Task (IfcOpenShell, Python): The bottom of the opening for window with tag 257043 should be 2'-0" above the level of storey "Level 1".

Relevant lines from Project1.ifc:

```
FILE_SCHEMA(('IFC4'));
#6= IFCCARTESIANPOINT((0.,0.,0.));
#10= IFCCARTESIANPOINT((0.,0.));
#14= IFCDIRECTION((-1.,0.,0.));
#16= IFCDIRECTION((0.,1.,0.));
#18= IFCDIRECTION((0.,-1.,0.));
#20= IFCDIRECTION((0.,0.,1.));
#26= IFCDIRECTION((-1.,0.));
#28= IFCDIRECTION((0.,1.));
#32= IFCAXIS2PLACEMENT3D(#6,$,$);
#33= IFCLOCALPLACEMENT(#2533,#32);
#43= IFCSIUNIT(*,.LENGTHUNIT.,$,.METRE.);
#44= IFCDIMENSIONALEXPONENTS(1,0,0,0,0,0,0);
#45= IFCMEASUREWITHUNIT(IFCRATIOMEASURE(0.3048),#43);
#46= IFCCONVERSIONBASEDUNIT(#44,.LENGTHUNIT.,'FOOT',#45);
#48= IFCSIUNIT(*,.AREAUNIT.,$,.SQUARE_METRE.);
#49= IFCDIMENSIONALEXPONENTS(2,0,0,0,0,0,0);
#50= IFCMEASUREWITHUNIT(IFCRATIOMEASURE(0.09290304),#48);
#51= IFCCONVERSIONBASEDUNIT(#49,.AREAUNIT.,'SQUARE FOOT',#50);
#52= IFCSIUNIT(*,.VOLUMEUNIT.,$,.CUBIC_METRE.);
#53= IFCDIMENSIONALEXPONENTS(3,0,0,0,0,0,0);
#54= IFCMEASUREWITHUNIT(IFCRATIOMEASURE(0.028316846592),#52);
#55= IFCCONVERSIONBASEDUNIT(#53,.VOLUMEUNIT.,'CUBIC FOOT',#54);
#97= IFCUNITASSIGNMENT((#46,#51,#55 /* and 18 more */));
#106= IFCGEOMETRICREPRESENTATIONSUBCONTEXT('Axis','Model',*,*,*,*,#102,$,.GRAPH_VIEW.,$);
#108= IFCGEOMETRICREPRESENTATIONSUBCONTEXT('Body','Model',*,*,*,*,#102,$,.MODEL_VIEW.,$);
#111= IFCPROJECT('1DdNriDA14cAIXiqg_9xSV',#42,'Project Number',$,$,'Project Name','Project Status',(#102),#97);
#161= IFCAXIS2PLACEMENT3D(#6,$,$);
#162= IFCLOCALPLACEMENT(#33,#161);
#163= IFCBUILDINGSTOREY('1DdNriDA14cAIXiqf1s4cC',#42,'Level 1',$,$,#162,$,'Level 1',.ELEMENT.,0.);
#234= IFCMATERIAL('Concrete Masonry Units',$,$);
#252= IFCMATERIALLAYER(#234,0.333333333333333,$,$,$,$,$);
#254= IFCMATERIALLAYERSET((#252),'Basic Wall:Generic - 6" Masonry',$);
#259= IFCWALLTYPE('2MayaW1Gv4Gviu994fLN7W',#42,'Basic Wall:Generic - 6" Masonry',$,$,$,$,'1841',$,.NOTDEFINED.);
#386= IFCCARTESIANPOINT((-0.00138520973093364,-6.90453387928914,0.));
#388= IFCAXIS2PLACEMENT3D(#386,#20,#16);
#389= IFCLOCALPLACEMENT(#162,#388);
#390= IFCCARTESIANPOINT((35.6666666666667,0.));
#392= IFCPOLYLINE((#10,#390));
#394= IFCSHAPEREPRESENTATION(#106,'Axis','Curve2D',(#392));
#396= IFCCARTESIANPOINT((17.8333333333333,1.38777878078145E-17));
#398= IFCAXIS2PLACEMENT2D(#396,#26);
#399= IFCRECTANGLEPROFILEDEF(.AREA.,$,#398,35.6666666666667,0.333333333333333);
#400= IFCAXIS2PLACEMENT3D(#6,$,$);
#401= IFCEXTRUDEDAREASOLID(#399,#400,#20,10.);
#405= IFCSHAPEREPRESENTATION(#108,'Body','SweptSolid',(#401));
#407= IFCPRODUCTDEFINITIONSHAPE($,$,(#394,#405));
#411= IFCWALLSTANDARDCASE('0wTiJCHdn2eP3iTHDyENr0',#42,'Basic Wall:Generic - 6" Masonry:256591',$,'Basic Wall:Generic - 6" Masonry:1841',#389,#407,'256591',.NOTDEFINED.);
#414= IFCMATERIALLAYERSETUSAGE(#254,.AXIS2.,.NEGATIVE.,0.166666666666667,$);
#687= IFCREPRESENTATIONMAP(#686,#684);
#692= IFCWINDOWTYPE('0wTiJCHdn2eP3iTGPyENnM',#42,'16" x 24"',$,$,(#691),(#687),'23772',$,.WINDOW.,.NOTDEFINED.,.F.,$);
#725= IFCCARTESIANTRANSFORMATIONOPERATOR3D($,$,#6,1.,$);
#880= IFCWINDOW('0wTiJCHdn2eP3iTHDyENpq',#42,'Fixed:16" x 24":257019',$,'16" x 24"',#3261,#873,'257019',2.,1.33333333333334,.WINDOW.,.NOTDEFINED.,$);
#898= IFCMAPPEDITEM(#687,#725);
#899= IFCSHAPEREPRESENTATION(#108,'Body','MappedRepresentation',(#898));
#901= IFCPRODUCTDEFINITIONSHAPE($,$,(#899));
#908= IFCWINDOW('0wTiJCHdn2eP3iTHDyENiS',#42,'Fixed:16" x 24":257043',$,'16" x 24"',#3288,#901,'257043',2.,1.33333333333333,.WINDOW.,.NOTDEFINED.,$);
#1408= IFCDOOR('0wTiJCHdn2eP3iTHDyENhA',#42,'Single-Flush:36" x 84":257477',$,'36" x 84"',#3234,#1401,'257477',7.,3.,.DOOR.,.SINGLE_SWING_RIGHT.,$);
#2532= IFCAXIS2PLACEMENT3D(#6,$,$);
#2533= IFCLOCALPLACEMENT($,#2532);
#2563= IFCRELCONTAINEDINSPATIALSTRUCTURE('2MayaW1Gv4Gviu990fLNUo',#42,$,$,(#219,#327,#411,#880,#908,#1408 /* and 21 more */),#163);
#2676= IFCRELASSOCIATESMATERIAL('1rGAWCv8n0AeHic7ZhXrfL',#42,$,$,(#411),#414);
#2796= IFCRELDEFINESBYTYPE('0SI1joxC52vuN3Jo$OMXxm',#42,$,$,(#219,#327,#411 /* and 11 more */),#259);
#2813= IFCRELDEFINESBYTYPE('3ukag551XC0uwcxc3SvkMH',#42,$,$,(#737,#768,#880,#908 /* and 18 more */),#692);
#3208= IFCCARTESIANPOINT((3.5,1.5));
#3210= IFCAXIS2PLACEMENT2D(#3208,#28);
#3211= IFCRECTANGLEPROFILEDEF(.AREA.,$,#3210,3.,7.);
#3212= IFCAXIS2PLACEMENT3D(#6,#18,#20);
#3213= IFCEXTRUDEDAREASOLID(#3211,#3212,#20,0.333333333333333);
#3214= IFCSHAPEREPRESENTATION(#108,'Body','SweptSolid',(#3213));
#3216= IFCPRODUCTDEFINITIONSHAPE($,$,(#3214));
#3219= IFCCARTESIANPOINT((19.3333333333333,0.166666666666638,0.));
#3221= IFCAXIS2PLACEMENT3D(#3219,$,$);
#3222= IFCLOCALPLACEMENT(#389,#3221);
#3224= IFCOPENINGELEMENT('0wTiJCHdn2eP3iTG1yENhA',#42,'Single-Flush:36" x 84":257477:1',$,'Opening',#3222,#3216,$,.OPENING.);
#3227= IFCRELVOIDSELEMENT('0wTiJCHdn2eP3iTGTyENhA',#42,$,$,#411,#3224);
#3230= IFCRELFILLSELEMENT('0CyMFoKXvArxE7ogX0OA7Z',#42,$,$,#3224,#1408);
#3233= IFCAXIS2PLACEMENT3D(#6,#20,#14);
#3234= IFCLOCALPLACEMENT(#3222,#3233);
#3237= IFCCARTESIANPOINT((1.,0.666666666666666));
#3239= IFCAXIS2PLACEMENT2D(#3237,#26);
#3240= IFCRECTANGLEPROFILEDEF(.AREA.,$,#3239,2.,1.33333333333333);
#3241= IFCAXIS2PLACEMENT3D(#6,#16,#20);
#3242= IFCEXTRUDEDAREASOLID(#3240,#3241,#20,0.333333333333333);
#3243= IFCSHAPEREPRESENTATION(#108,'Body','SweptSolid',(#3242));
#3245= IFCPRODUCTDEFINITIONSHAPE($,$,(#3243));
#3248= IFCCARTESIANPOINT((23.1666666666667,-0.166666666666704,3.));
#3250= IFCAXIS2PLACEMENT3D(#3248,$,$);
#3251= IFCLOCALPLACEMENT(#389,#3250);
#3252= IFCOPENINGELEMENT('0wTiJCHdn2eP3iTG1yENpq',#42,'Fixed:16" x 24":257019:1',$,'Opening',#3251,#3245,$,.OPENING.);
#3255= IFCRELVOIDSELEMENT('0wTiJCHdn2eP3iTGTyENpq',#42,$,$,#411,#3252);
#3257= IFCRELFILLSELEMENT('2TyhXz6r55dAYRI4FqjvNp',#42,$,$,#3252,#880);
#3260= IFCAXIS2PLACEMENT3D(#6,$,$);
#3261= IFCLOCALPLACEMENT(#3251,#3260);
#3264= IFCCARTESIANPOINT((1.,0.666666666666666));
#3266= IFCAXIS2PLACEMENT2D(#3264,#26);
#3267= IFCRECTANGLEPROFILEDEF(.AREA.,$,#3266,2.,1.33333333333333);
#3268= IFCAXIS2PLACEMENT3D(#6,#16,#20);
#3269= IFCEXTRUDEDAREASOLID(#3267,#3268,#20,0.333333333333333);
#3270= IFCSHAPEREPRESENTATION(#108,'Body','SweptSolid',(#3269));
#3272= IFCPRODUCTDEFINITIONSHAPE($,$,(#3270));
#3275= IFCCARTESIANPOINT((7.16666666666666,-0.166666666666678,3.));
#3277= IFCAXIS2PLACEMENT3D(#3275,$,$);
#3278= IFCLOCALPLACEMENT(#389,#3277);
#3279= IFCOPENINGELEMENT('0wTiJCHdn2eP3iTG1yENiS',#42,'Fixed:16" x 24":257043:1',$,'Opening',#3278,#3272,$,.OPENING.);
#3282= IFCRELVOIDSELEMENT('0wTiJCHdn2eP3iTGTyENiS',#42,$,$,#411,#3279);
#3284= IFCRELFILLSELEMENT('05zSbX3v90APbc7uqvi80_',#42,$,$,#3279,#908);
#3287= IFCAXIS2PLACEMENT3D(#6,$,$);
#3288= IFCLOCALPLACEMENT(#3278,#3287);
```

```python
import numpy as np
import ifcopenshell
import ifcopenshell.api.geometry
import ifcopenshell.geom
import ifcopenshell.util.element
import ifcopenshell.util.placement
import ifcopenshell.util.shape
import ifcopenshell.util.unit

model = ifcopenshell.open("Project1.ifc")
unit_scale = ifcopenshell.util.unit.calculate_unit_scale(model)

window = model.by_id(908)
opening = window.FillsVoids[0].RelatingOpeningElement
storey = ifcopenshell.util.element.get_container(window, ifc_class="IfcBuildingStorey")
level = ifcopenshell.util.placement.get_local_placement(storey.ObjectPlacement)[2, 3]

# The opening's origin need not be at the sill, so measure its lowest point.
shape = ifcopenshell.geom.create_shape(ifcopenshell.geom.settings(), opening)
bottom = ifcopenshell.util.shape.get_shape_bottom_elevation(shape, shape.geometry) / unit_scale
dz = level + 24 * 0.0254 / unit_scale - bottom

shift = np.array([0.0, 0.0, dz])
# The window is placed relative to its opening, so it follows when the opening moves.
matrix = ifcopenshell.util.placement.get_local_placement(opening.ObjectPlacement)
matrix[:3, 3] += shift
ifcopenshell.api.geometry.edit_object_placement(
    model, product=opening, matrix=matrix, is_si=False, should_transform_children=True
)

print(f"moved by {dz * unit_scale:+.3f} m")

model.write("Project1_edited.ifc")
```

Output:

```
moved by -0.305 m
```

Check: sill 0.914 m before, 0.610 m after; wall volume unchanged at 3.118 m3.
